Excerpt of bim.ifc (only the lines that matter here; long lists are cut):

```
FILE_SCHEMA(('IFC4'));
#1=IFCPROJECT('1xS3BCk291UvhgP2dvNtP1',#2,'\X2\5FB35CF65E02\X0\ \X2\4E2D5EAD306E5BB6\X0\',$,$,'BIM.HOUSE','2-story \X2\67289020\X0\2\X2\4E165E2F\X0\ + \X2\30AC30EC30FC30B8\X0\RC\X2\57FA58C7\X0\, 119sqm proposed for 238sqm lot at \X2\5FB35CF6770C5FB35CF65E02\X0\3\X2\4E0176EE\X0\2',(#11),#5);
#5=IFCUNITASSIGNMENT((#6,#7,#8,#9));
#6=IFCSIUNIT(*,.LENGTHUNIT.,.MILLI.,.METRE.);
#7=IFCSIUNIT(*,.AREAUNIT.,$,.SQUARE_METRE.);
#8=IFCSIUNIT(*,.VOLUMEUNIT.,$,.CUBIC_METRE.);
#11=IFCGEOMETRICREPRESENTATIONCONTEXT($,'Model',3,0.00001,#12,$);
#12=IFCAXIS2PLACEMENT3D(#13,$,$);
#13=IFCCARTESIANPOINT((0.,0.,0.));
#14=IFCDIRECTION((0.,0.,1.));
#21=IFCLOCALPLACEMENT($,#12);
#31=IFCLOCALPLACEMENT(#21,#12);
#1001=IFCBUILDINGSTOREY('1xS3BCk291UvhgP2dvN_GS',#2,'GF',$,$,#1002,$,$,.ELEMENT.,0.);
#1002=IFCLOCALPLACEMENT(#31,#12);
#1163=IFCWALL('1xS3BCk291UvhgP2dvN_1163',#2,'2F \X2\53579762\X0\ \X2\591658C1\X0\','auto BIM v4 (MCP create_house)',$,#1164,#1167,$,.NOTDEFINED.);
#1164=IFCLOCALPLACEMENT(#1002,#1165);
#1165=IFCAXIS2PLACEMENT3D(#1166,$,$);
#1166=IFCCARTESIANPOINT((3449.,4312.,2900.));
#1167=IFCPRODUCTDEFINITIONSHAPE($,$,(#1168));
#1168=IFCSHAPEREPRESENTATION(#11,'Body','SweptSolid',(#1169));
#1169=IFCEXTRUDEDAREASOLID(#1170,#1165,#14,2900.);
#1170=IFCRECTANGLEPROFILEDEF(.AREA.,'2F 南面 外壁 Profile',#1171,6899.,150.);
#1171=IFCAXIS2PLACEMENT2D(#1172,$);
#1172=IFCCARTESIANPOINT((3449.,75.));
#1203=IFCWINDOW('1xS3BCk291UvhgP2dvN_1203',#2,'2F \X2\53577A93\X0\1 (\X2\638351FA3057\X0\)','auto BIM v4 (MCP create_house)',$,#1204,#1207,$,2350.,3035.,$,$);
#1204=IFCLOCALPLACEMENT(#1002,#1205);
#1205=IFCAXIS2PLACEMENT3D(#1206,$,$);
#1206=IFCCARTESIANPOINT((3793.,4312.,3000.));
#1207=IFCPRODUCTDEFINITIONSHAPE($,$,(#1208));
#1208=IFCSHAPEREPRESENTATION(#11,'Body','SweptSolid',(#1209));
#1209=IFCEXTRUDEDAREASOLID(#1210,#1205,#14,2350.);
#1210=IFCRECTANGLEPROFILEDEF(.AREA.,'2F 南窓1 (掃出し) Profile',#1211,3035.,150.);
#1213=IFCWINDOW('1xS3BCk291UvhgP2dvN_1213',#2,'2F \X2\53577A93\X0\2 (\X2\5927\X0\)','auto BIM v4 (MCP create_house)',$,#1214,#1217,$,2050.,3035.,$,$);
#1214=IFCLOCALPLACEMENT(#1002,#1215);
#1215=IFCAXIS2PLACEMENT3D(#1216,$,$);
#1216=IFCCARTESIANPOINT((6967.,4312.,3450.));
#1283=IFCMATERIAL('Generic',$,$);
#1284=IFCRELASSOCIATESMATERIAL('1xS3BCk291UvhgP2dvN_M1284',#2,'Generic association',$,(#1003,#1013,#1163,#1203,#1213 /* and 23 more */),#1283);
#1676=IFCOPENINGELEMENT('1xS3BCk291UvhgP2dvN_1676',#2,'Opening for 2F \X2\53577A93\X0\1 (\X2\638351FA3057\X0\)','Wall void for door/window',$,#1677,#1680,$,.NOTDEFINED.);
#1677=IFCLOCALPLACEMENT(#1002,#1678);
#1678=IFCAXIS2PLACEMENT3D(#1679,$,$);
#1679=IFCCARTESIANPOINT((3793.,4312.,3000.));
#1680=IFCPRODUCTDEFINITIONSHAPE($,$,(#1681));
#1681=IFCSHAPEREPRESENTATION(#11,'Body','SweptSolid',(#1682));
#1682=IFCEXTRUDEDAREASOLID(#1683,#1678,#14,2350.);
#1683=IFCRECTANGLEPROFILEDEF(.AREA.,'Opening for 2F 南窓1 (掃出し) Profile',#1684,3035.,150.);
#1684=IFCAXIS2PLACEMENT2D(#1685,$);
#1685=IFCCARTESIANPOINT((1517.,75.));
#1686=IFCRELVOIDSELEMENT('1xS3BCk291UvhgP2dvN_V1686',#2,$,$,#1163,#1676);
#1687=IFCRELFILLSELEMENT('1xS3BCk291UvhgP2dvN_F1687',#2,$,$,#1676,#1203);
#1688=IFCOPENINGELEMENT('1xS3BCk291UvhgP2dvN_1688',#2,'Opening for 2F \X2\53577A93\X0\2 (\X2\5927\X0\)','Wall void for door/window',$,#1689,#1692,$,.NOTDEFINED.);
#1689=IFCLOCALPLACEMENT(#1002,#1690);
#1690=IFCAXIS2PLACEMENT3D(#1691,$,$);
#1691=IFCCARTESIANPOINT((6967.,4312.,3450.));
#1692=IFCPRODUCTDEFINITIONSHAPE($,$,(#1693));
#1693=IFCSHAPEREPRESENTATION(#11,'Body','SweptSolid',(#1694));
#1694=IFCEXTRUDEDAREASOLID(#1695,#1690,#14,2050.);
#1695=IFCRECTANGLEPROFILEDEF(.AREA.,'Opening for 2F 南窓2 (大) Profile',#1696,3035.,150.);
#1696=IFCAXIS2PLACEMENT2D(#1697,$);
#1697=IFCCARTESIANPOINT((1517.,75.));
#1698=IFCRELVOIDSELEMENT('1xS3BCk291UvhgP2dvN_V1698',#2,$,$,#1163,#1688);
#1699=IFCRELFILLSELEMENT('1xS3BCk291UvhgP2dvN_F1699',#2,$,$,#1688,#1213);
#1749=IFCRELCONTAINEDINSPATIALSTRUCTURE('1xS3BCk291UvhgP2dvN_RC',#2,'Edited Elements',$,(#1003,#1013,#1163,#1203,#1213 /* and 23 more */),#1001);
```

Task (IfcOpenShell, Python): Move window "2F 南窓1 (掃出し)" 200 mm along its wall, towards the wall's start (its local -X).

```python
import ifcopenshell
import ifcopenshell.api.geometry
import ifcopenshell.util.placement

model = ifcopenshell.open("bim.ifc")

window = model.by_guid("1xS3BCk291UvhgP2dvN_1203")
opening = window.FillsVoids[0].RelatingOpeningElement
wall = opening.VoidsElements[0].RelatingBuildingElement

wall_matrix = ifcopenshell.util.placement.get_local_placement(wall.ObjectPlacement)
shift = wall_matrix[:3, 0] * -200.0
before = ifcopenshell.util.placement.get_local_placement(window.ObjectPlacement)[:3, 3].copy()

# The window is not placed relative to its opening, so move both.
for product in (opening, window):
    matrix = ifcopenshell.util.placement.get_local_placement(product.ObjectPlacement)
    matrix[:3, 3] += shift
    ifcopenshell.api.geometry.edit_object_placement(model, product=product, matrix=matrix, is_si=False)

after = ifcopenshell.util.placement.get_local_placement(window.ObjectPlacement)[:3, 3]
print("window moved by", (after - before).round(3) + 0.0)

model.write("bim_edited.ifc")
```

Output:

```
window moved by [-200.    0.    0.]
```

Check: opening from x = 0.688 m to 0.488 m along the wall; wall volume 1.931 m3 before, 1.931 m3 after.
